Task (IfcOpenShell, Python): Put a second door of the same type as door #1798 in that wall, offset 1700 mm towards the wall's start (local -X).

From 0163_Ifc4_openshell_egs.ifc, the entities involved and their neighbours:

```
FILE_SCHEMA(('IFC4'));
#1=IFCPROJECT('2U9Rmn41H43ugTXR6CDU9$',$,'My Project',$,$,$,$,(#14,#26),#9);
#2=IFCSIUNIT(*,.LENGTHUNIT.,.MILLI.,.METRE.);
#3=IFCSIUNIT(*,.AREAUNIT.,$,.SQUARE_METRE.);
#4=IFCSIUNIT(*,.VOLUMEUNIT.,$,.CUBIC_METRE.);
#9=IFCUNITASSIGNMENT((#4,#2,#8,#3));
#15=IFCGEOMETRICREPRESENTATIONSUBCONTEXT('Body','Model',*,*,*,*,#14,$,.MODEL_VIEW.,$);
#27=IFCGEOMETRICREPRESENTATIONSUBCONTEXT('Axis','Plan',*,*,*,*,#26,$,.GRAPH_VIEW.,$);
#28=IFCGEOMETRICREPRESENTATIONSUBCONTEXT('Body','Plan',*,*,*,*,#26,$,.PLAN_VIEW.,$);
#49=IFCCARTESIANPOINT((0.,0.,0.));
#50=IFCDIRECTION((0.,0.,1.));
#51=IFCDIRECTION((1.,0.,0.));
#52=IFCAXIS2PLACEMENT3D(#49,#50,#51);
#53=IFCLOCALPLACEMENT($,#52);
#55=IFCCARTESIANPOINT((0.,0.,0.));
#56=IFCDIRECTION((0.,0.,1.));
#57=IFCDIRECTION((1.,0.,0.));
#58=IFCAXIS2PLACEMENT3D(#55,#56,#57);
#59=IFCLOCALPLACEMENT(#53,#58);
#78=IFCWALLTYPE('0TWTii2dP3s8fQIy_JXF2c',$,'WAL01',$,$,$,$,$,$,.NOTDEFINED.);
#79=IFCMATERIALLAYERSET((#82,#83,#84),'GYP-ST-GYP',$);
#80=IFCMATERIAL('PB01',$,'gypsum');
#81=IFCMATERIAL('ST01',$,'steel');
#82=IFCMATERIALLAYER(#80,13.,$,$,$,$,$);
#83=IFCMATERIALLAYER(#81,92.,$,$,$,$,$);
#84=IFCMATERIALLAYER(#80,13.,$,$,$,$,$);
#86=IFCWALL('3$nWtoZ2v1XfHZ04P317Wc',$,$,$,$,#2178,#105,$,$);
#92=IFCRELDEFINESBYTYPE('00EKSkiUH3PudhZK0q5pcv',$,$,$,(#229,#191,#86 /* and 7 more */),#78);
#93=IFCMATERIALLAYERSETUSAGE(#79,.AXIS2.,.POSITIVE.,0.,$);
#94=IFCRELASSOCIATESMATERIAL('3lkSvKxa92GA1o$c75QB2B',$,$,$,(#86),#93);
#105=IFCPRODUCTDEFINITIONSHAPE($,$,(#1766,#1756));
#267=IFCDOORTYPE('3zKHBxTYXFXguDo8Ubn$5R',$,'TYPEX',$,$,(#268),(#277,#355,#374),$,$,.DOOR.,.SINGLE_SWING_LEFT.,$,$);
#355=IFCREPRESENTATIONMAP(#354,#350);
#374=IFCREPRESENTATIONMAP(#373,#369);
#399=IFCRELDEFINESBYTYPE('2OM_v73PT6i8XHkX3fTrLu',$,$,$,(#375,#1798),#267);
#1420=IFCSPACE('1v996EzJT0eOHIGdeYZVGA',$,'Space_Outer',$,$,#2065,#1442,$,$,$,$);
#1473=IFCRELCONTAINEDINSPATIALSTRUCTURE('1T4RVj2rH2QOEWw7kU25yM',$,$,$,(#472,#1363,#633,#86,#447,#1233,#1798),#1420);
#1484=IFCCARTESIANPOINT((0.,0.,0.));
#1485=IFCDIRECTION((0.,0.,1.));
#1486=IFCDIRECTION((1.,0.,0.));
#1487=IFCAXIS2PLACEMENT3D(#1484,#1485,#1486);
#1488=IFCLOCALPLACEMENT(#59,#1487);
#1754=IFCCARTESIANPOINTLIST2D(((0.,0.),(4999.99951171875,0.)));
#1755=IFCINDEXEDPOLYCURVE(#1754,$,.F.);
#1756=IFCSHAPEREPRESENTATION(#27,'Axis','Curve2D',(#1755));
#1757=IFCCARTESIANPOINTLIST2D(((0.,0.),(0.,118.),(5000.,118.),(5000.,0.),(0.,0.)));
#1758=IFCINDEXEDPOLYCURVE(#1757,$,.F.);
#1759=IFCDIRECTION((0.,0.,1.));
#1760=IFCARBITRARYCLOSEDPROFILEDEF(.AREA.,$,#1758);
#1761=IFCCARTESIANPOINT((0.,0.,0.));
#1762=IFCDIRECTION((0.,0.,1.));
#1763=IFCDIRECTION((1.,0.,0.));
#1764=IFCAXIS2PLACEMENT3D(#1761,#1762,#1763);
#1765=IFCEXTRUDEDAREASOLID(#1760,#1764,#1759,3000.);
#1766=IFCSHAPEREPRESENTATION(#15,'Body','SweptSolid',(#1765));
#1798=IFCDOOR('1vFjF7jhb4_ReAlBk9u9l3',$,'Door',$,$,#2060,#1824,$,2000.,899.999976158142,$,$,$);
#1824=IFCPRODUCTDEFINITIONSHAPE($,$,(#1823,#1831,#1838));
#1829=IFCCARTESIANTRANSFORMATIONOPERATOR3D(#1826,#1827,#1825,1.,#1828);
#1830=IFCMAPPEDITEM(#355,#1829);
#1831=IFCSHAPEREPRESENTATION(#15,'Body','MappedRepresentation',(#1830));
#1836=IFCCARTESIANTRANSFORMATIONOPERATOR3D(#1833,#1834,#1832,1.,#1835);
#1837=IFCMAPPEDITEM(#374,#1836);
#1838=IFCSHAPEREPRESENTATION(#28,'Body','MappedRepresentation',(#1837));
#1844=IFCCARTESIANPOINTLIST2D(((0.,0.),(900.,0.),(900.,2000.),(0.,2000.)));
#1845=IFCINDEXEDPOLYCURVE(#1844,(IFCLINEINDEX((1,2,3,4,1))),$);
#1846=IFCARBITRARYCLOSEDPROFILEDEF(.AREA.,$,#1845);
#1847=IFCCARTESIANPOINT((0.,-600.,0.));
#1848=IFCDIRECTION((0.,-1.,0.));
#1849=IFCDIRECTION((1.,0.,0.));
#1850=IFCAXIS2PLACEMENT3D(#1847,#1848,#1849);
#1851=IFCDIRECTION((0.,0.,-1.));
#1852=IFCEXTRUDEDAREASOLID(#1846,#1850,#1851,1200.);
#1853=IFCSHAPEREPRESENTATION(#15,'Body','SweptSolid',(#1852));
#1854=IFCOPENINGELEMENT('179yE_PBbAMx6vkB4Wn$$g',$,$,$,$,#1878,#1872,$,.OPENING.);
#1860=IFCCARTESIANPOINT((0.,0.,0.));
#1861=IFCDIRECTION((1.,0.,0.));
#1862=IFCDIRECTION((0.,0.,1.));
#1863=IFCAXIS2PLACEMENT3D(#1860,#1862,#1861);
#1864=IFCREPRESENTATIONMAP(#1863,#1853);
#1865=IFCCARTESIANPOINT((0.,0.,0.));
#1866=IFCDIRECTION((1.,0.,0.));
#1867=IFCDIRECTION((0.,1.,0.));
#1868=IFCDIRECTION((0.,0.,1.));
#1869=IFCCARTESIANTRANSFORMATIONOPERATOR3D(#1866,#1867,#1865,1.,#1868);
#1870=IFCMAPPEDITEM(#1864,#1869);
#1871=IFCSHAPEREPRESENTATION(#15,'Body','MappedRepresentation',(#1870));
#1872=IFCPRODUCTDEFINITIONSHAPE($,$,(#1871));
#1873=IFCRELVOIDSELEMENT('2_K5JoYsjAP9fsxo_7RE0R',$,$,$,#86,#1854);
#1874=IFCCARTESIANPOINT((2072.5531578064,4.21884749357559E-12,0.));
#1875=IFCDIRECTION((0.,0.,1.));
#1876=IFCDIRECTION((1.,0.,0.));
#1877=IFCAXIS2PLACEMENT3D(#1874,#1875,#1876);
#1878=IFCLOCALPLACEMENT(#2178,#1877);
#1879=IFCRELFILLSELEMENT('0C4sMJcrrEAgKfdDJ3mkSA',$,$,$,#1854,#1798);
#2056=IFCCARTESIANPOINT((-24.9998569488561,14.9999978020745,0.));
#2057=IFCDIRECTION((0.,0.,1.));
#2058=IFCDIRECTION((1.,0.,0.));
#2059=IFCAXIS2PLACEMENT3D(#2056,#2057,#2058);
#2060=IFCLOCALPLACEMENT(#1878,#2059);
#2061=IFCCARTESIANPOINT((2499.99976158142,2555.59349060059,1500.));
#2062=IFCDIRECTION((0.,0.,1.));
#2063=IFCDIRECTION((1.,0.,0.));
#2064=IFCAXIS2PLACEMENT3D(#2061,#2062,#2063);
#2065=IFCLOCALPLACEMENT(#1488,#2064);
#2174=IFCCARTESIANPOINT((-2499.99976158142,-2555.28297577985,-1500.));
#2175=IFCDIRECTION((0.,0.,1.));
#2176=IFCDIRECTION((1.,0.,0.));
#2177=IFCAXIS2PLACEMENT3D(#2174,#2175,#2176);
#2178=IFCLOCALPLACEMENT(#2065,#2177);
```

```python
import ifcopenshell
import ifcopenshell.api.feature
import ifcopenshell.api.geometry
import ifcopenshell.api.root
import ifcopenshell.geom
import ifcopenshell.util.element
import ifcopenshell.util.placement
import ifcopenshell.util.shape

model = ifcopenshell.open("0163_Ifc4_openshell_egs.ifc")
settings = ifcopenshell.geom.settings()


def volume(element):
    """Net volume in cubic metres, openings subtracted."""
    shape = ifcopenshell.geom.create_shape(settings, element)
    return ifcopenshell.util.shape.get_volume(shape.geometry)


door = model.by_guid("1vFjF7jhb4_ReAlBk9u9l3")
opening = door.FillsVoids[0].RelatingOpeningElement
wall = opening.VoidsElements[0].RelatingBuildingElement
before = volume(wall)
shift = ifcopenshell.util.placement.get_local_placement(wall.ObjectPlacement)[:3, 0] * -1700.0

# copy_class copies the void relationship, type, container and properties, but no geometry.
new_opening = ifcopenshell.api.root.copy_class(model, product=opening)
new_opening.Representation = ifcopenshell.util.element.copy_deep(
    model, opening.Representation, exclude=["IfcGeometricRepresentationContext", "IfcRepresentationMap"]
)
new_door = ifcopenshell.api.root.copy_class(model, product=door)
new_door.Representation = ifcopenshell.util.element.copy_deep(
    model, door.Representation, exclude=["IfcGeometricRepresentationContext", "IfcRepresentationMap"]
)
ifcopenshell.api.feature.add_filling(model, opening=new_opening, element=new_door)

for old, new in ((opening, new_opening), (door, new_door)):
    matrix = ifcopenshell.util.placement.get_local_placement(old.ObjectPlacement)
    matrix[:3, 3] += shift
    ifcopenshell.api.geometry.edit_object_placement(model, product=new, matrix=matrix, is_si=False)

after = volume(wall)

print(f"wall volume {before:.3f} -> {after:.3f} m3")

model.write("0163_Ifc4_openshell_egs-out.ifc")
```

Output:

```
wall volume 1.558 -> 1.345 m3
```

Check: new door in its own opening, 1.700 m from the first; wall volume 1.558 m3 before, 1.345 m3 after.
